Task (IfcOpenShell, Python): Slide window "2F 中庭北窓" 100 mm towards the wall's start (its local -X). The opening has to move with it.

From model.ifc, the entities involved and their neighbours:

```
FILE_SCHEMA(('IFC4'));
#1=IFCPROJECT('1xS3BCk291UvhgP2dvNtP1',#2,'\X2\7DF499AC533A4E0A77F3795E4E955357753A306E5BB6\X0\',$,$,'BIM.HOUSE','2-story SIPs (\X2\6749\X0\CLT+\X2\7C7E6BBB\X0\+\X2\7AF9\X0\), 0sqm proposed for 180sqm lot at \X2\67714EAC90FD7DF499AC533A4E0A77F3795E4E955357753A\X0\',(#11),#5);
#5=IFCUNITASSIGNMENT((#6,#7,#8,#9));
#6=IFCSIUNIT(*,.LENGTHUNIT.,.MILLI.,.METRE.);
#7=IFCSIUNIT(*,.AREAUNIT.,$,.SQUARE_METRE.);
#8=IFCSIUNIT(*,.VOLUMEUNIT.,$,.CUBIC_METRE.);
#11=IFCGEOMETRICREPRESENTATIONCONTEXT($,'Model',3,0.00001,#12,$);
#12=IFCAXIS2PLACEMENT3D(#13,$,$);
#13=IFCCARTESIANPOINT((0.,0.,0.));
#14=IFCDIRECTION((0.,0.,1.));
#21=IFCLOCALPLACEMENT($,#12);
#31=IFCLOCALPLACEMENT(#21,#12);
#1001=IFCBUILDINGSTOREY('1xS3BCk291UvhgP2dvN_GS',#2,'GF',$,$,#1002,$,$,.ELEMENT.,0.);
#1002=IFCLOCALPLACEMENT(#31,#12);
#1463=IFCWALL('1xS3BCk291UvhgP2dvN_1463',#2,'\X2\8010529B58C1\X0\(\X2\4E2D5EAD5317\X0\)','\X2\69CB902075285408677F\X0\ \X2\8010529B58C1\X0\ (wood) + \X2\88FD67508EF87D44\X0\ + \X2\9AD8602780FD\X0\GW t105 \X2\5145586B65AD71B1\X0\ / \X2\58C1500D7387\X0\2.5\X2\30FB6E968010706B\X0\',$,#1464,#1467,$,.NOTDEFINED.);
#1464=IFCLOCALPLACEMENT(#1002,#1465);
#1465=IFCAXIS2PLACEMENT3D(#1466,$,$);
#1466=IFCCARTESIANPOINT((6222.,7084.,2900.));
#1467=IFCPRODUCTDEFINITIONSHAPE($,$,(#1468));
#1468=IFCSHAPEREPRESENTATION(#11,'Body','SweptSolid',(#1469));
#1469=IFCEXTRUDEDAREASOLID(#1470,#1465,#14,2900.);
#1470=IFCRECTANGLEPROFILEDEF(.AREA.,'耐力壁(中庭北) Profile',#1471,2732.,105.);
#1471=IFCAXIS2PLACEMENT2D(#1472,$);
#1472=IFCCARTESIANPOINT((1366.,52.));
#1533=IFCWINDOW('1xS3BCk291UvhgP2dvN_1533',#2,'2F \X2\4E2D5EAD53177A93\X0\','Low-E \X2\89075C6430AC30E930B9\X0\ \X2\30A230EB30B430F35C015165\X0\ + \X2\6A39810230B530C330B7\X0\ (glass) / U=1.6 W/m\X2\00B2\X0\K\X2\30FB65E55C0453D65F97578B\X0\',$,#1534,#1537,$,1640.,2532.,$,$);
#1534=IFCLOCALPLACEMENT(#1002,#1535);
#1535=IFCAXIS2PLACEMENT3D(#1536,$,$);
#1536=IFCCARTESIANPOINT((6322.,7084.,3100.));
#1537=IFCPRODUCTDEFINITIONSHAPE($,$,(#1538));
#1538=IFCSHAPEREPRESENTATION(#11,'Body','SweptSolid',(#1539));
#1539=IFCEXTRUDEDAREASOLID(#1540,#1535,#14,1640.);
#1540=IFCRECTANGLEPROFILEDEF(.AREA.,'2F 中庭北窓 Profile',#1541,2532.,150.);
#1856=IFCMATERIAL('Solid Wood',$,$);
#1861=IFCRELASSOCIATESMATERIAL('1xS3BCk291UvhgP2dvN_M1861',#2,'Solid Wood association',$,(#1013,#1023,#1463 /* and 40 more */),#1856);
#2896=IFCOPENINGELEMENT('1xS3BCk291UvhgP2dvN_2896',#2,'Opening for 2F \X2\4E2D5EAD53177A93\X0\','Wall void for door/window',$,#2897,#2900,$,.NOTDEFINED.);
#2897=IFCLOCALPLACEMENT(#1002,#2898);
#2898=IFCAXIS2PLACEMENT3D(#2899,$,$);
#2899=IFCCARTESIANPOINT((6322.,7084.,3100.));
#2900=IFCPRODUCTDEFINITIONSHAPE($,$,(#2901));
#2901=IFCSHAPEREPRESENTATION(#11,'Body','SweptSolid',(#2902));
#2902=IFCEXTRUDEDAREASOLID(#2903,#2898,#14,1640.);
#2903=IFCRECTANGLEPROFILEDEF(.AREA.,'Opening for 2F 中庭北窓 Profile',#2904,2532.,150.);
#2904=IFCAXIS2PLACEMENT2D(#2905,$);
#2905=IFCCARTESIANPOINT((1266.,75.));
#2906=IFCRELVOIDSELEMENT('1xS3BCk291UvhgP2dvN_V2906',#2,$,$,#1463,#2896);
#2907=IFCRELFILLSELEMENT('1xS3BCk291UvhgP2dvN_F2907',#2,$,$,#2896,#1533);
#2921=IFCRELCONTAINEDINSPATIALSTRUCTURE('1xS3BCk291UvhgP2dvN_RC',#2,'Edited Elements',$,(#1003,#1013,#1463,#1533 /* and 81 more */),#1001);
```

```python
import ifcopenshell
import ifcopenshell.api.geometry
import ifcopenshell.util.placement

model = ifcopenshell.open("model.ifc")

window = model.by_guid("1xS3BCk291UvhgP2dvN_1533")
opening = window.FillsVoids[0].RelatingOpeningElement
wall = opening.VoidsElements[0].RelatingBuildingElement

wall_matrix = ifcopenshell.util.placement.get_local_placement(wall.ObjectPlacement)
shift = wall_matrix[:3, 0] * -100.0
before = ifcopenshell.util.placement.get_local_placement(window.ObjectPlacement)[:3, 3].copy()

# The window is not placed relative to its opening, so move both.
for product in (opening, window):
    matrix = ifcopenshell.util.placement.get_local_placement(product.ObjectPlacement)
    matrix[:3, 3] += shift
    ifcopenshell.api.geometry.edit_object_placement(model, product=product, matrix=matrix, is_si=False)

after = ifcopenshell.util.placement.get_local_placement(window.ObjectPlacement)[:3, 3]
print("window moved by", (after - before).round(3) + 0.0)

model.write("model-out.ifc")
```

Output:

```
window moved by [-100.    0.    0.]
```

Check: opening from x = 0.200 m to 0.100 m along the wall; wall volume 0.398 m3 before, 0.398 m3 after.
